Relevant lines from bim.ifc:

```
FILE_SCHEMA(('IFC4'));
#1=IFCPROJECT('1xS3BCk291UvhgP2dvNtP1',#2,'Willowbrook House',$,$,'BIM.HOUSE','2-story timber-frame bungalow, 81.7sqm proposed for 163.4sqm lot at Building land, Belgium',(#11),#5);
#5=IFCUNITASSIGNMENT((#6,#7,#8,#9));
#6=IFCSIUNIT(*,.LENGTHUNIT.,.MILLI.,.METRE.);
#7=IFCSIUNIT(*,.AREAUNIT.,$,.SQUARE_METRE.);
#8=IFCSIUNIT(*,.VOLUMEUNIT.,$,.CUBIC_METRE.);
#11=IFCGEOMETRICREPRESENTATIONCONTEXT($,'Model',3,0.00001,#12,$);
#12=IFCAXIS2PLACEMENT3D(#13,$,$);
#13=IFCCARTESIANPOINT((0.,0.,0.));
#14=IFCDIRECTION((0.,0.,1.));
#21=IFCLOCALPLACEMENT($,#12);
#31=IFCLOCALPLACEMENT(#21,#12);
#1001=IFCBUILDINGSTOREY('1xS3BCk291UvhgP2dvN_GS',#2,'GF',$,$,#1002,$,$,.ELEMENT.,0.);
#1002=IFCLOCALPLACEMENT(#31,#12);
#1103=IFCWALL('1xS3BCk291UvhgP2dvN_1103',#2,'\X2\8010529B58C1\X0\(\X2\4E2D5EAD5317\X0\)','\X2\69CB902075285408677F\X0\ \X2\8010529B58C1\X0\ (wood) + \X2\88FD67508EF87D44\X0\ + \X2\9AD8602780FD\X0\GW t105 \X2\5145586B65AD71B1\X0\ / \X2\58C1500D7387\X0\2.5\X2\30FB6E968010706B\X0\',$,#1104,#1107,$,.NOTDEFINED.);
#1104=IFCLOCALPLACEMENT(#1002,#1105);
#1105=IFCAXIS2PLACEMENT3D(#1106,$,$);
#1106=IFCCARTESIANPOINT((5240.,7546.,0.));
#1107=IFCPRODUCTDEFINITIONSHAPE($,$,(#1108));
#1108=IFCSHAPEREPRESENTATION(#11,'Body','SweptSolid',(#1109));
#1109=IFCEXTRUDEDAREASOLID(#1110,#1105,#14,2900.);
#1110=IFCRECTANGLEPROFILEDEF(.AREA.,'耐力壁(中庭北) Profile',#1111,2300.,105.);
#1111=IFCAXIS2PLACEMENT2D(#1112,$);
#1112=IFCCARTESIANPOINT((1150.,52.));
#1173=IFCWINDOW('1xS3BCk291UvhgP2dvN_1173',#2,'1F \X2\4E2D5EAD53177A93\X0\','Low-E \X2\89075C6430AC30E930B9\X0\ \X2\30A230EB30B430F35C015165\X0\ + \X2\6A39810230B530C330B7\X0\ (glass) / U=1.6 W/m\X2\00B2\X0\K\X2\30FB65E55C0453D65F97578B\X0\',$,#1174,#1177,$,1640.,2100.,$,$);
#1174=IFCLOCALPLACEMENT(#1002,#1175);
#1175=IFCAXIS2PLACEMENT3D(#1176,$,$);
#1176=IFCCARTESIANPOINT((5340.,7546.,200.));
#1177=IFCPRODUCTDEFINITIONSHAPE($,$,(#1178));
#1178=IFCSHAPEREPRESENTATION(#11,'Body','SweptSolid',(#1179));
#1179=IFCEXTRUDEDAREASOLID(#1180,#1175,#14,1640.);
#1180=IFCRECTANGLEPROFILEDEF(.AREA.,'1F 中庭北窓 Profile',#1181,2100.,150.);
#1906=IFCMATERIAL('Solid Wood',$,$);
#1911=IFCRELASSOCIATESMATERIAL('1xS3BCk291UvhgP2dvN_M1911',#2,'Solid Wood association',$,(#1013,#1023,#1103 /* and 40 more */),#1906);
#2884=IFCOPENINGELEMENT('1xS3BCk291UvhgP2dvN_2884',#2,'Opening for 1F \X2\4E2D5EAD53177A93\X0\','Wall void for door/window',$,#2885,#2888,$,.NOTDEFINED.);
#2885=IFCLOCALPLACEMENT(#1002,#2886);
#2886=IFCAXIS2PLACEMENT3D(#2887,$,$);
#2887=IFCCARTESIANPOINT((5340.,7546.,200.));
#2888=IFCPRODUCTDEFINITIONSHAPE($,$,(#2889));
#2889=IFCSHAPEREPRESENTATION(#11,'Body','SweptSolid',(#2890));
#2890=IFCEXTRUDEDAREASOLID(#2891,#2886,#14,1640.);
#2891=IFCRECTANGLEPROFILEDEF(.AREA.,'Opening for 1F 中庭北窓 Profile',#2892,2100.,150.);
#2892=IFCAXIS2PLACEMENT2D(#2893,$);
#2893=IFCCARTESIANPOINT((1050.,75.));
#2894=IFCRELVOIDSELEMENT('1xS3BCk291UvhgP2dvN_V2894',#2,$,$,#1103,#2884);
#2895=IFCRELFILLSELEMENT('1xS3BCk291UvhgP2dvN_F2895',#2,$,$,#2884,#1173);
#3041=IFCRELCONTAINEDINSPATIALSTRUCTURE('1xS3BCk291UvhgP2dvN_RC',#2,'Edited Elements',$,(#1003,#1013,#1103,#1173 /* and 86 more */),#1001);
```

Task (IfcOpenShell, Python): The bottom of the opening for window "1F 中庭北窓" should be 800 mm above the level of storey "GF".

```python
import numpy as np
import ifcopenshell
import ifcopenshell.api.geometry
import ifcopenshell.geom
import ifcopenshell.util.element
import ifcopenshell.util.placement
import ifcopenshell.util.shape
import ifcopenshell.util.unit

model = ifcopenshell.open("bim.ifc")
unit_scale = ifcopenshell.util.unit.calculate_unit_scale(model)

window = model.by_guid("1xS3BCk291UvhgP2dvN_1173")
opening = window.FillsVoids[0].RelatingOpeningElement
storey = ifcopenshell.util.element.get_container(window, ifc_class="IfcBuildingStorey")
level = ifcopenshell.util.placement.get_local_placement(storey.ObjectPlacement)[2, 3]

# The opening's origin need not be at the sill, so measure its lowest point.
shape = ifcopenshell.geom.create_shape(ifcopenshell.geom.settings(), opening)
bottom = ifcopenshell.util.shape.get_shape_bottom_elevation(shape, shape.geometry) / unit_scale
dz = level + 0.8 / unit_scale - bottom

shift = np.array([0.0, 0.0, dz])
# The window is not placed relative to its opening, so move both.
for product in (opening, window):
    matrix = ifcopenshell.util.placement.get_local_placement(product.ObjectPlacement)
    matrix[:3, 3] += shift
    ifcopenshell.api.geometry.edit_object_placement(model, product=product, matrix=matrix, is_si=False)

print(f"moved by {dz * unit_scale:+.3f} m")

model.write("bim_edited.ifc")
```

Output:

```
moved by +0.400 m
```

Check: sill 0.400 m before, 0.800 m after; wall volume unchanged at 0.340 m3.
